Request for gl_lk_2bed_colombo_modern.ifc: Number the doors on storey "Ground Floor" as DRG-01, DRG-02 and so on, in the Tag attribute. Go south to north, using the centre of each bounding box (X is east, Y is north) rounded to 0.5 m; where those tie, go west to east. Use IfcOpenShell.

First a look at what the model holds.

```python
import ifcopenshell
import ifcopenshell.util.element
import ifcopenshell.util.placement

model = ifcopenshell.open("gl_lk_2bed_colombo_modern.ifc")
print(model.schema)
storey = next(s for s in model.by_type("IfcBuildingStorey") if s.Name == "Ground Floor")
doors = [e for e in ifcopenshell.util.element.get_decomposition(storey) if e.is_a("IfcDoor")]
for e in sorted(doors, key=lambda e: e.id()):
    origin = ifcopenshell.util.placement.get_local_placement(e.ObjectPlacement)[:3, 3]
    print(e.id(), e.Tag, e.Name, origin.round(2) + 0.0, sep=" | ")
```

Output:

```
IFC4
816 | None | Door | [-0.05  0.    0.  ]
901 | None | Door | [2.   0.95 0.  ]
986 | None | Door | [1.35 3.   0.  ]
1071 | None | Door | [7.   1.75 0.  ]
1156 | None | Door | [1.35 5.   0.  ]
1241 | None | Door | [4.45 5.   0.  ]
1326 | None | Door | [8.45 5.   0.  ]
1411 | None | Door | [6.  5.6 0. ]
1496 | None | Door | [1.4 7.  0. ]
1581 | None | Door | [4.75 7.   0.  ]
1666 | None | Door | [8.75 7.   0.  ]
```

```python
import ifcopenshell
import ifcopenshell.geom
import ifcopenshell.util.element
import ifcopenshell.util.shape

model = ifcopenshell.open("gl_lk_2bed_colombo_modern.ifc")
settings = ifcopenshell.geom.settings()
settings.set("use-world-coords", True)


def centre(element):
    shape = ifcopenshell.geom.create_shape(settings, element)
    return ifcopenshell.util.shape.get_bbox_centroid(shape.geometry)


storey = next(s for s in model.by_type("IfcBuildingStorey") if s.Name == "Ground Floor")
doors = [e for e in ifcopenshell.util.element.get_decomposition(storey) if e.is_a("IfcDoor")]

# Insertion points can sit at a corner or the storey origin, so sort by the geometry (in metres).
centres = {e: centre(e) for e in doors}
doors.sort(key=lambda e: (round(centres[e][1] / 0.5), centres[e][0]))

for i, e in enumerate(doors, start=1):
    number = f"DRG-{i:02d}"
    e.Tag = number
    print(e.id(), number)

model.write("gl_lk_2bed_colombo_modern_updated.ifc")
```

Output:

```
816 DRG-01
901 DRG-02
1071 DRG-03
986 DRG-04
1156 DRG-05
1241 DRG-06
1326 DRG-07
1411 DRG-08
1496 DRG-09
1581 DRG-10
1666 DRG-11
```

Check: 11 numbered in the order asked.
